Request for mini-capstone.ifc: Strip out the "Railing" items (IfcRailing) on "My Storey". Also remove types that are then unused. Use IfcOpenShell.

First a look at what the model holds.

```python
import ifcopenshell
import ifcopenshell.util.element

model = ifcopenshell.open("mini-capstone.ifc")
print(model.schema)
storey = next(s for s in model.by_type("IfcBuildingStorey") if s.Name == "My Storey")
railings = [e for e in ifcopenshell.util.element.get_decomposition(storey) if e.is_a("IfcRailing")]
seen = {}
for e in railings:
    element_type = ifcopenshell.util.element.get_type(e)
    name = element_type.Name if element_type not in (None, e) else None
    seen[name] = seen.get(name, 0) + 1
for name, count in sorted(seen.items(), key=str):
    print(count, "x", name)
```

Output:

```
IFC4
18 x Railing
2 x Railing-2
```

```python
import ifcopenshell
import ifcopenshell.api.root
import ifcopenshell.util.element

model = ifcopenshell.open("mini-capstone.ifc")

storey = next(s for s in model.by_type("IfcBuildingStorey") if s.Name == "My Storey")
railings = [e for e in ifcopenshell.util.element.get_decomposition(storey) if e.is_a("IfcRailing")]
targets = [e for e in railings if (t := ifcopenshell.util.element.get_type(e)) not in (None, e) and t.Name == "Railing"]
types = {ifcopenshell.util.element.get_type(e) for e in targets} - {None, *targets}

for e in targets:
    ifcopenshell.api.root.remove_product(model, product=e)
print(len(targets), "removed")

unused = [t for t in types if not ifcopenshell.util.element.get_types(t)]
for t in unused:
    ifcopenshell.api.root.remove_product(model, product=t)
print(len(unused), "unused types removed")

model.write("mini-capstone_updated.ifc")
```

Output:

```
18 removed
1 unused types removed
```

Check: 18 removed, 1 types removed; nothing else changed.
